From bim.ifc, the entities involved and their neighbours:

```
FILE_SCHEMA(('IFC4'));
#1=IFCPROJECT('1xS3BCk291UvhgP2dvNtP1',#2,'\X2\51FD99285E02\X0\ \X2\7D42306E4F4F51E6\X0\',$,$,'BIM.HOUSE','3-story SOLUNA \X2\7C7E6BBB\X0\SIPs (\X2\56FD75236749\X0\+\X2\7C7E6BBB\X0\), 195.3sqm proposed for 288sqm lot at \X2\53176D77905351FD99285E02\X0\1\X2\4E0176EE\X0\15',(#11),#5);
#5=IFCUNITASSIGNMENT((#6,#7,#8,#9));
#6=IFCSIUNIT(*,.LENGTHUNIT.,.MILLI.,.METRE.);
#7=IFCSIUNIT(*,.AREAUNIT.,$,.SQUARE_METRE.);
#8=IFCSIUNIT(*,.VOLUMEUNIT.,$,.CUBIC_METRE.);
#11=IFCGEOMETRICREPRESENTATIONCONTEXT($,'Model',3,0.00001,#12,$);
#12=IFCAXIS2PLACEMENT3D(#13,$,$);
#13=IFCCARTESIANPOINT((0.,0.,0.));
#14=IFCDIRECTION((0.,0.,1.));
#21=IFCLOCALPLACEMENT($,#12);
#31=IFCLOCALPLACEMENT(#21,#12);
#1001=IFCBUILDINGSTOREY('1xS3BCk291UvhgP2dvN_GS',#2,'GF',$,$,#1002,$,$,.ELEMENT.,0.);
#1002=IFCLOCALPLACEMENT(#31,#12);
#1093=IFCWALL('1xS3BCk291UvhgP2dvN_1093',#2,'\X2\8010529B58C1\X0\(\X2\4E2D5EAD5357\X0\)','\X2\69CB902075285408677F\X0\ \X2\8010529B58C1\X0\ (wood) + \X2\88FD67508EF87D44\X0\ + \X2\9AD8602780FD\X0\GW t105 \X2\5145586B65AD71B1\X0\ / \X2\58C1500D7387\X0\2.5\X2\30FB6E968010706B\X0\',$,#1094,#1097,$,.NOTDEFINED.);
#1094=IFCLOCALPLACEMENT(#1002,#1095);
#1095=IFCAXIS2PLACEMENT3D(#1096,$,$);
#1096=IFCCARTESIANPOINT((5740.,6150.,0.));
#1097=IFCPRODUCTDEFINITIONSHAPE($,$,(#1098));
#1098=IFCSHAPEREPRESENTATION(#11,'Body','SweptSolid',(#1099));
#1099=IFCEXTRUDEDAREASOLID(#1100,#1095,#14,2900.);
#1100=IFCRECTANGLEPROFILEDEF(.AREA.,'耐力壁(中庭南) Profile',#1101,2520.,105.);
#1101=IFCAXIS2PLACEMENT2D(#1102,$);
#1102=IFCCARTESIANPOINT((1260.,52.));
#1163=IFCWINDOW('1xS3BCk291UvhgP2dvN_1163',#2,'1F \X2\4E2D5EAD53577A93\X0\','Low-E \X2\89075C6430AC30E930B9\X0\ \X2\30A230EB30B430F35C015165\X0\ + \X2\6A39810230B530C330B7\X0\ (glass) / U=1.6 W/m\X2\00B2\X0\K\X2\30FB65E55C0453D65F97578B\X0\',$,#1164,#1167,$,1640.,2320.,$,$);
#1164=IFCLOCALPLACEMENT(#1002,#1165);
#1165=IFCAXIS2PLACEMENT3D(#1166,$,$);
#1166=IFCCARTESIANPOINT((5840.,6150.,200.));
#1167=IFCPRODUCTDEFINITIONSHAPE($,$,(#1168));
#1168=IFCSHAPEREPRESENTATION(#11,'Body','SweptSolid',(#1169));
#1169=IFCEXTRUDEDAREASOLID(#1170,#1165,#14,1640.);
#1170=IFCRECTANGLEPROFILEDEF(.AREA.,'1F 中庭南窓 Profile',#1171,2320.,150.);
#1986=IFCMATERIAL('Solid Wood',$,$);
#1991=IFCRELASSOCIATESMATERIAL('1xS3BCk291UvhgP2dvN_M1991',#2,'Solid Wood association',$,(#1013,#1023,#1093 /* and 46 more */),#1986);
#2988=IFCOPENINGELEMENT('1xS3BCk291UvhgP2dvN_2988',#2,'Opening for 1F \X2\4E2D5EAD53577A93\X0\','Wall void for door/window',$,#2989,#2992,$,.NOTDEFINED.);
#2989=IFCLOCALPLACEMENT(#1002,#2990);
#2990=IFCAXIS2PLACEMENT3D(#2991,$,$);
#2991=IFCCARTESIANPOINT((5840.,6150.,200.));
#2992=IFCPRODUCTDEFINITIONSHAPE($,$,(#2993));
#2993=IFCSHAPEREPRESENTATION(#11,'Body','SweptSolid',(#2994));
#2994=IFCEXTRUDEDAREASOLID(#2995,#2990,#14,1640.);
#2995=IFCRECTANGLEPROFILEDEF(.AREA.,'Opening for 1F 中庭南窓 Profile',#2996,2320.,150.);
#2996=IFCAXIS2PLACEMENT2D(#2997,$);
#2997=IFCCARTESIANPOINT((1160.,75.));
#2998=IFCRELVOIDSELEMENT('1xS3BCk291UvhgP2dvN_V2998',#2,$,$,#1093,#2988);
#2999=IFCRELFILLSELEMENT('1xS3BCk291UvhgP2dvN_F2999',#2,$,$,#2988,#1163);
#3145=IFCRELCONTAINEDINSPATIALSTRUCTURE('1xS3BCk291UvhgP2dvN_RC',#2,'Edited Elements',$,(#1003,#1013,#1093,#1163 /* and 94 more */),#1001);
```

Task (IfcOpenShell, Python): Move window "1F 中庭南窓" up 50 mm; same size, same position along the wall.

```python
import numpy as np
import ifcopenshell
import ifcopenshell.api.geometry
import ifcopenshell.util.placement
import ifcopenshell.util.unit

model = ifcopenshell.open("bim.ifc")
unit_scale = ifcopenshell.util.unit.calculate_unit_scale(model)

window = model.by_guid("1xS3BCk291UvhgP2dvN_1163")
opening = window.FillsVoids[0].RelatingOpeningElement
dz = 50.0

shift = np.array([0.0, 0.0, dz])
# The window is not placed relative to its opening, so move both.
for product in (opening, window):
    matrix = ifcopenshell.util.placement.get_local_placement(product.ObjectPlacement)
    matrix[:3, 3] += shift
    ifcopenshell.api.geometry.edit_object_placement(model, product=product, matrix=matrix, is_si=False)

print(f"moved by {dz * unit_scale:+.3f} m")

model.write("bim_edited.ifc")
```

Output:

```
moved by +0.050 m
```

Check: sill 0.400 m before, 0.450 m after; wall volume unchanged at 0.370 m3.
